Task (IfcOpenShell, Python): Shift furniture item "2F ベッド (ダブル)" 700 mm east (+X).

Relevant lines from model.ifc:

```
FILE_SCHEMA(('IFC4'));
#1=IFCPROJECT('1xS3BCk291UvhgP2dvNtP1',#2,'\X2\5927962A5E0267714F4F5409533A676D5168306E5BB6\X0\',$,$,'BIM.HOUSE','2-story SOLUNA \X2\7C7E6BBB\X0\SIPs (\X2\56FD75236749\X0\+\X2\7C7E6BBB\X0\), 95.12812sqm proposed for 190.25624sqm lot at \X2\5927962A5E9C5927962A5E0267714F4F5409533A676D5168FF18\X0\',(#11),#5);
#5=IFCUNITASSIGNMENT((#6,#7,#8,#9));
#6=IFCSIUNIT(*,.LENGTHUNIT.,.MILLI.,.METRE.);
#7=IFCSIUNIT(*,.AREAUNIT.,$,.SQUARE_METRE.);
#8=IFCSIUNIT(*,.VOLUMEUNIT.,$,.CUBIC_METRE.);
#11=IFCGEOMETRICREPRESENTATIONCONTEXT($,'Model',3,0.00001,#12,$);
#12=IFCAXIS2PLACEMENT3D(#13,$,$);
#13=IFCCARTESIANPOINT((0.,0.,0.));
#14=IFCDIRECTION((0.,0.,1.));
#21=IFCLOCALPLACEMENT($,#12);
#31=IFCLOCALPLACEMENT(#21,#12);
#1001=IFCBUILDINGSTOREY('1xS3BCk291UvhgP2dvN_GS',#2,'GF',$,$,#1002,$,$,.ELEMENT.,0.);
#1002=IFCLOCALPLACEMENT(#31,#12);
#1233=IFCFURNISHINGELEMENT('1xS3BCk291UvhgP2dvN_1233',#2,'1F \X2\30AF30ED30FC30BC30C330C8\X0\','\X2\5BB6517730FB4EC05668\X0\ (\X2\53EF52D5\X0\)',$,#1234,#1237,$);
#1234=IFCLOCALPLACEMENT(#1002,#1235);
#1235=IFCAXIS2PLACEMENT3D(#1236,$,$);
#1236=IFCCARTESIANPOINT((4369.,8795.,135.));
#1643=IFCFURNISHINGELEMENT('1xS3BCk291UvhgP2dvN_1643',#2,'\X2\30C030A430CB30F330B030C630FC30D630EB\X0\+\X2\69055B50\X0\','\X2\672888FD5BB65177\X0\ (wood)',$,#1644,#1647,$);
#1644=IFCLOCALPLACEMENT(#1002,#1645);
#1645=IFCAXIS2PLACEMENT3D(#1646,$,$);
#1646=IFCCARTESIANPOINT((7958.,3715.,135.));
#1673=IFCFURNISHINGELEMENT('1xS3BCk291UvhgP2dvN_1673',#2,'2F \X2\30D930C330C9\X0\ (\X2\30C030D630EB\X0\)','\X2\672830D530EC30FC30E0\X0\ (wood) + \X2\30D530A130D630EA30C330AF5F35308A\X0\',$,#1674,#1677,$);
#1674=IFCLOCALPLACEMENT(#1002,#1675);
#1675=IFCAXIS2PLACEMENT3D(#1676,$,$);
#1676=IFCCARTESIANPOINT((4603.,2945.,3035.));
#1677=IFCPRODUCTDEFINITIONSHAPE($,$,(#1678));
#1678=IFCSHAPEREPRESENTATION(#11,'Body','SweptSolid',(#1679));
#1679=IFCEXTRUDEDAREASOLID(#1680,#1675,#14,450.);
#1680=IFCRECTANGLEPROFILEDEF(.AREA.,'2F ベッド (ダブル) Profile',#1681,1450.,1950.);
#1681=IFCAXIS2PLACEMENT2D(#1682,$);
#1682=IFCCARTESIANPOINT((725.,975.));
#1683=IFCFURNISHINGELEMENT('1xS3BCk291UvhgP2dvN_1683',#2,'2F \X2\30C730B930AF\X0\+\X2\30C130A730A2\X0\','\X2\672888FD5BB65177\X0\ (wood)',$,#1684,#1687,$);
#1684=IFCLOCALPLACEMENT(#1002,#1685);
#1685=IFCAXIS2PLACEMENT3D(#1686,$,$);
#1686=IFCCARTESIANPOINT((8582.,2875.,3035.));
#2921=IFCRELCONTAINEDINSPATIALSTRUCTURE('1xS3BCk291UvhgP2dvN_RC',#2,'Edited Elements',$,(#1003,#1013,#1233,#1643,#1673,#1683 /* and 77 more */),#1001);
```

```python
import ifcopenshell
import ifcopenshell.api.geometry
import ifcopenshell.util.placement
import ifcopenshell.util.unit

model = ifcopenshell.open("model.ifc")
unit_scale = ifcopenshell.util.unit.calculate_unit_scale(model)

item = model.by_id(1673)
matrix = ifcopenshell.util.placement.get_local_placement(item.ObjectPlacement)
matrix[0, 3] += 0.7 / unit_scale
ifcopenshell.api.geometry.edit_object_placement(model, product=item, matrix=matrix, is_si=False)

print(ifcopenshell.util.placement.get_local_placement(item.ObjectPlacement).round(3) + 0.0)

model.write("model_rev.ifc")
```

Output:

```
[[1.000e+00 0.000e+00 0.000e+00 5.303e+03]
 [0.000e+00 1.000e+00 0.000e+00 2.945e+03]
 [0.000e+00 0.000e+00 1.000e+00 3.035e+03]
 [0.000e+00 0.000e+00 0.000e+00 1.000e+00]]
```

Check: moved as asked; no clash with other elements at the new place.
